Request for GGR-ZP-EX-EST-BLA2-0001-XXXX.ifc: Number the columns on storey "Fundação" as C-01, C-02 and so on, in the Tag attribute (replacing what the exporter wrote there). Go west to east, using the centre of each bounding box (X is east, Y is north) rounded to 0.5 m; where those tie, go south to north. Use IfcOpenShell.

First a look at what the model holds.

```python
import ifcopenshell
import ifcopenshell.util.element
import ifcopenshell.util.placement

model = ifcopenshell.open("GGR-ZP-EX-EST-BLA2-0001-XXXX.ifc")
print(model.schema)
storey = next(s for s in model.by_type("IfcBuildingStorey") if s.Name == "Fundação")
columns = [e for e in ifcopenshell.util.element.get_decomposition(storey) if e.is_a("IfcColumn")]
for e in sorted(columns, key=lambda e: e.id()):
    origin = ifcopenshell.util.placement.get_local_placement(e.ObjectPlacement)[:3, 3]
    print(e.id(), e.Tag, e.Name, origin.round(2) + 0.0, sep=" | ")
```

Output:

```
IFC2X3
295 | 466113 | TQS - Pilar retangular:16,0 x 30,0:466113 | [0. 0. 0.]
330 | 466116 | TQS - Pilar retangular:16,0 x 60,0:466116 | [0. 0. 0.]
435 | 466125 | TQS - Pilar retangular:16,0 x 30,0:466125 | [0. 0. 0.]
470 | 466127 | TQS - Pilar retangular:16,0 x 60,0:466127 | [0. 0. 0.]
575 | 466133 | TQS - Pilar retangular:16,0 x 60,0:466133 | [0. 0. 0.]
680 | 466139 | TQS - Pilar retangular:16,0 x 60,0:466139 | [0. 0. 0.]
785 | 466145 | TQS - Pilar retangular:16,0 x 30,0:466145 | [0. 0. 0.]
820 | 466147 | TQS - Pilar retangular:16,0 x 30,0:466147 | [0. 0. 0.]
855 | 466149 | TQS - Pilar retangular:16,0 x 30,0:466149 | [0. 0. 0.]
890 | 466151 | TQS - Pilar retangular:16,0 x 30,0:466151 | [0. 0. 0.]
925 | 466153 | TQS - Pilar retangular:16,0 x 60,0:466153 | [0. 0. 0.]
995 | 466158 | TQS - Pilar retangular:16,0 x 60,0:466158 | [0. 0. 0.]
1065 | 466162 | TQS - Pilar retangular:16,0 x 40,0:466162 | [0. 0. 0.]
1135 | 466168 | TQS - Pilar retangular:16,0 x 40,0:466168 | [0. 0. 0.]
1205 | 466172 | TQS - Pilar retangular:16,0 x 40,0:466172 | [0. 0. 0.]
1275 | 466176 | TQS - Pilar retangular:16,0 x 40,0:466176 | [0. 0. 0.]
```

```python
import ifcopenshell
import ifcopenshell.geom
import ifcopenshell.util.element
import ifcopenshell.util.shape

model = ifcopenshell.open("GGR-ZP-EX-EST-BLA2-0001-XXXX.ifc")
settings = ifcopenshell.geom.settings()
settings.set("use-world-coords", True)


def centre(element):
    shape = ifcopenshell.geom.create_shape(settings, element)
    return ifcopenshell.util.shape.get_bbox_centroid(shape.geometry)


storey = next(s for s in model.by_type("IfcBuildingStorey") if s.Name == "Fundação")
columns = [e for e in ifcopenshell.util.element.get_decomposition(storey) if e.is_a("IfcColumn")]

# Insertion points can sit at a corner or the storey origin, so sort by the geometry (in metres).
centres = {e: centre(e) for e in columns}
columns.sort(key=lambda e: (round(centres[e][0] / 0.5), centres[e][1]))

for i, e in enumerate(columns, start=1):
    number = f"C-{i:02d}"
    e.Tag = number
    print(e.id(), number)

model.write("GGR-ZP-EX-EST-BLA2-0001-XXXX_v2.ifc")
```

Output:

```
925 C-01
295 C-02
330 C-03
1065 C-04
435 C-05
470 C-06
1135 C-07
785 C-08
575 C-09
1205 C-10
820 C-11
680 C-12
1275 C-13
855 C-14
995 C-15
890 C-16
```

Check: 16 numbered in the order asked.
